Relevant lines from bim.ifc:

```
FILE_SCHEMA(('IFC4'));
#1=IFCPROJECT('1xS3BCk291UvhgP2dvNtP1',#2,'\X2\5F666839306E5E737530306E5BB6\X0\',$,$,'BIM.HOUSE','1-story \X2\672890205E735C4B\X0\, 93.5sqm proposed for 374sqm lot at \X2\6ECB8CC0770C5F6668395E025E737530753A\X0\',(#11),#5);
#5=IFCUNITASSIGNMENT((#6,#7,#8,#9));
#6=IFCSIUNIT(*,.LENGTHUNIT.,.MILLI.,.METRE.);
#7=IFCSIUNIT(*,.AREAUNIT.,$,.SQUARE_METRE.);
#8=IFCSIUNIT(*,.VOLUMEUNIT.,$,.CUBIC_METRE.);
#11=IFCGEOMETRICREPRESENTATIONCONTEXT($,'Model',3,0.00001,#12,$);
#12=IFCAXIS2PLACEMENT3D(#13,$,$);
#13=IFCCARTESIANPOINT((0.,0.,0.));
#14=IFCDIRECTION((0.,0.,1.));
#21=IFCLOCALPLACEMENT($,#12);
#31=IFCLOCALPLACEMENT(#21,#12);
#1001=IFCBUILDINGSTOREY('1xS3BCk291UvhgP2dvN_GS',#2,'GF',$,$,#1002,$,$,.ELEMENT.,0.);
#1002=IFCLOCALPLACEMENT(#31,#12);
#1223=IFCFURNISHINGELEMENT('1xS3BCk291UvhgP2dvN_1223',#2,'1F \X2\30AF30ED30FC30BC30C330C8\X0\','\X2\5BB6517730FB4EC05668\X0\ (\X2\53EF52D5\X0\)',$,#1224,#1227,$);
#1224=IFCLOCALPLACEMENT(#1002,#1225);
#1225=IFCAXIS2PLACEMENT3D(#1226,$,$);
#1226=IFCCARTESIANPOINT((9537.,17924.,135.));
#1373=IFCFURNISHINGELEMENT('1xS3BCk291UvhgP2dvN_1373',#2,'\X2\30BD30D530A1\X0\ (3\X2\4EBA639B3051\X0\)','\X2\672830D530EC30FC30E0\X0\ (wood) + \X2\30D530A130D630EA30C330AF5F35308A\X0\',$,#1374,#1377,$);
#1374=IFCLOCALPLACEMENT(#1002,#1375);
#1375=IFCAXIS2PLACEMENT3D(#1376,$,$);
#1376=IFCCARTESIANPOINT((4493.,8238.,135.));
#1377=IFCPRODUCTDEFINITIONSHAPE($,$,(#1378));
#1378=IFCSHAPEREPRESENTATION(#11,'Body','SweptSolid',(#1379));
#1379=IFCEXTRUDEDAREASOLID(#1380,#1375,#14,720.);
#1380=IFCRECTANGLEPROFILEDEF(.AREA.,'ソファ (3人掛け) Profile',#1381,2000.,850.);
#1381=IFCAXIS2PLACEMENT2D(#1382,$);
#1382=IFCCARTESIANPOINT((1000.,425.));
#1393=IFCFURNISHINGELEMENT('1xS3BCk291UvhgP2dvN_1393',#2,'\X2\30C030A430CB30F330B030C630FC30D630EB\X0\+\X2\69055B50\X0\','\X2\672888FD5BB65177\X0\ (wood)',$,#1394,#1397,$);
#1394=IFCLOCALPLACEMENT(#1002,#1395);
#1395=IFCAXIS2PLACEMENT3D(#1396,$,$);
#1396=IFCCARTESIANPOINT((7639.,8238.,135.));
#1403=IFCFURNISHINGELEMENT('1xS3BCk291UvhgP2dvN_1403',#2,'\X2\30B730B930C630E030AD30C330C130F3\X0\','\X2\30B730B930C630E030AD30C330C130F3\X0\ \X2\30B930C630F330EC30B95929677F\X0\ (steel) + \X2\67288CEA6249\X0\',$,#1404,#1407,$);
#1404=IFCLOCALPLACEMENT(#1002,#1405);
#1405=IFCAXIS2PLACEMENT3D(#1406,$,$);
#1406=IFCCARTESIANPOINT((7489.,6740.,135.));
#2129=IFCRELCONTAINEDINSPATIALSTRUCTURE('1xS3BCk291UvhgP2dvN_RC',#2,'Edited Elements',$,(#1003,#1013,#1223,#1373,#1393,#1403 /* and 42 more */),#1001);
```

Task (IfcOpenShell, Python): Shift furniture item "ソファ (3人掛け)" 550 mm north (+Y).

```python
import ifcopenshell
import ifcopenshell.api.geometry
import ifcopenshell.util.placement
import ifcopenshell.util.unit

model = ifcopenshell.open("bim.ifc")
unit_scale = ifcopenshell.util.unit.calculate_unit_scale(model)

item = model.by_id(1373)
matrix = ifcopenshell.util.placement.get_local_placement(item.ObjectPlacement)
matrix[1, 3] += 0.55 / unit_scale
ifcopenshell.api.geometry.edit_object_placement(model, product=item, matrix=matrix, is_si=False)

print(ifcopenshell.util.placement.get_local_placement(item.ObjectPlacement).round(3) + 0.0)

model.write("bim-out.ifc")
```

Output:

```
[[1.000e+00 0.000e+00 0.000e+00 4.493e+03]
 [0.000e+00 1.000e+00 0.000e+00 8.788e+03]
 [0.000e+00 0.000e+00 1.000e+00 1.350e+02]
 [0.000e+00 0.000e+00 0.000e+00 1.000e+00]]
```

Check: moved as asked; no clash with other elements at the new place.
